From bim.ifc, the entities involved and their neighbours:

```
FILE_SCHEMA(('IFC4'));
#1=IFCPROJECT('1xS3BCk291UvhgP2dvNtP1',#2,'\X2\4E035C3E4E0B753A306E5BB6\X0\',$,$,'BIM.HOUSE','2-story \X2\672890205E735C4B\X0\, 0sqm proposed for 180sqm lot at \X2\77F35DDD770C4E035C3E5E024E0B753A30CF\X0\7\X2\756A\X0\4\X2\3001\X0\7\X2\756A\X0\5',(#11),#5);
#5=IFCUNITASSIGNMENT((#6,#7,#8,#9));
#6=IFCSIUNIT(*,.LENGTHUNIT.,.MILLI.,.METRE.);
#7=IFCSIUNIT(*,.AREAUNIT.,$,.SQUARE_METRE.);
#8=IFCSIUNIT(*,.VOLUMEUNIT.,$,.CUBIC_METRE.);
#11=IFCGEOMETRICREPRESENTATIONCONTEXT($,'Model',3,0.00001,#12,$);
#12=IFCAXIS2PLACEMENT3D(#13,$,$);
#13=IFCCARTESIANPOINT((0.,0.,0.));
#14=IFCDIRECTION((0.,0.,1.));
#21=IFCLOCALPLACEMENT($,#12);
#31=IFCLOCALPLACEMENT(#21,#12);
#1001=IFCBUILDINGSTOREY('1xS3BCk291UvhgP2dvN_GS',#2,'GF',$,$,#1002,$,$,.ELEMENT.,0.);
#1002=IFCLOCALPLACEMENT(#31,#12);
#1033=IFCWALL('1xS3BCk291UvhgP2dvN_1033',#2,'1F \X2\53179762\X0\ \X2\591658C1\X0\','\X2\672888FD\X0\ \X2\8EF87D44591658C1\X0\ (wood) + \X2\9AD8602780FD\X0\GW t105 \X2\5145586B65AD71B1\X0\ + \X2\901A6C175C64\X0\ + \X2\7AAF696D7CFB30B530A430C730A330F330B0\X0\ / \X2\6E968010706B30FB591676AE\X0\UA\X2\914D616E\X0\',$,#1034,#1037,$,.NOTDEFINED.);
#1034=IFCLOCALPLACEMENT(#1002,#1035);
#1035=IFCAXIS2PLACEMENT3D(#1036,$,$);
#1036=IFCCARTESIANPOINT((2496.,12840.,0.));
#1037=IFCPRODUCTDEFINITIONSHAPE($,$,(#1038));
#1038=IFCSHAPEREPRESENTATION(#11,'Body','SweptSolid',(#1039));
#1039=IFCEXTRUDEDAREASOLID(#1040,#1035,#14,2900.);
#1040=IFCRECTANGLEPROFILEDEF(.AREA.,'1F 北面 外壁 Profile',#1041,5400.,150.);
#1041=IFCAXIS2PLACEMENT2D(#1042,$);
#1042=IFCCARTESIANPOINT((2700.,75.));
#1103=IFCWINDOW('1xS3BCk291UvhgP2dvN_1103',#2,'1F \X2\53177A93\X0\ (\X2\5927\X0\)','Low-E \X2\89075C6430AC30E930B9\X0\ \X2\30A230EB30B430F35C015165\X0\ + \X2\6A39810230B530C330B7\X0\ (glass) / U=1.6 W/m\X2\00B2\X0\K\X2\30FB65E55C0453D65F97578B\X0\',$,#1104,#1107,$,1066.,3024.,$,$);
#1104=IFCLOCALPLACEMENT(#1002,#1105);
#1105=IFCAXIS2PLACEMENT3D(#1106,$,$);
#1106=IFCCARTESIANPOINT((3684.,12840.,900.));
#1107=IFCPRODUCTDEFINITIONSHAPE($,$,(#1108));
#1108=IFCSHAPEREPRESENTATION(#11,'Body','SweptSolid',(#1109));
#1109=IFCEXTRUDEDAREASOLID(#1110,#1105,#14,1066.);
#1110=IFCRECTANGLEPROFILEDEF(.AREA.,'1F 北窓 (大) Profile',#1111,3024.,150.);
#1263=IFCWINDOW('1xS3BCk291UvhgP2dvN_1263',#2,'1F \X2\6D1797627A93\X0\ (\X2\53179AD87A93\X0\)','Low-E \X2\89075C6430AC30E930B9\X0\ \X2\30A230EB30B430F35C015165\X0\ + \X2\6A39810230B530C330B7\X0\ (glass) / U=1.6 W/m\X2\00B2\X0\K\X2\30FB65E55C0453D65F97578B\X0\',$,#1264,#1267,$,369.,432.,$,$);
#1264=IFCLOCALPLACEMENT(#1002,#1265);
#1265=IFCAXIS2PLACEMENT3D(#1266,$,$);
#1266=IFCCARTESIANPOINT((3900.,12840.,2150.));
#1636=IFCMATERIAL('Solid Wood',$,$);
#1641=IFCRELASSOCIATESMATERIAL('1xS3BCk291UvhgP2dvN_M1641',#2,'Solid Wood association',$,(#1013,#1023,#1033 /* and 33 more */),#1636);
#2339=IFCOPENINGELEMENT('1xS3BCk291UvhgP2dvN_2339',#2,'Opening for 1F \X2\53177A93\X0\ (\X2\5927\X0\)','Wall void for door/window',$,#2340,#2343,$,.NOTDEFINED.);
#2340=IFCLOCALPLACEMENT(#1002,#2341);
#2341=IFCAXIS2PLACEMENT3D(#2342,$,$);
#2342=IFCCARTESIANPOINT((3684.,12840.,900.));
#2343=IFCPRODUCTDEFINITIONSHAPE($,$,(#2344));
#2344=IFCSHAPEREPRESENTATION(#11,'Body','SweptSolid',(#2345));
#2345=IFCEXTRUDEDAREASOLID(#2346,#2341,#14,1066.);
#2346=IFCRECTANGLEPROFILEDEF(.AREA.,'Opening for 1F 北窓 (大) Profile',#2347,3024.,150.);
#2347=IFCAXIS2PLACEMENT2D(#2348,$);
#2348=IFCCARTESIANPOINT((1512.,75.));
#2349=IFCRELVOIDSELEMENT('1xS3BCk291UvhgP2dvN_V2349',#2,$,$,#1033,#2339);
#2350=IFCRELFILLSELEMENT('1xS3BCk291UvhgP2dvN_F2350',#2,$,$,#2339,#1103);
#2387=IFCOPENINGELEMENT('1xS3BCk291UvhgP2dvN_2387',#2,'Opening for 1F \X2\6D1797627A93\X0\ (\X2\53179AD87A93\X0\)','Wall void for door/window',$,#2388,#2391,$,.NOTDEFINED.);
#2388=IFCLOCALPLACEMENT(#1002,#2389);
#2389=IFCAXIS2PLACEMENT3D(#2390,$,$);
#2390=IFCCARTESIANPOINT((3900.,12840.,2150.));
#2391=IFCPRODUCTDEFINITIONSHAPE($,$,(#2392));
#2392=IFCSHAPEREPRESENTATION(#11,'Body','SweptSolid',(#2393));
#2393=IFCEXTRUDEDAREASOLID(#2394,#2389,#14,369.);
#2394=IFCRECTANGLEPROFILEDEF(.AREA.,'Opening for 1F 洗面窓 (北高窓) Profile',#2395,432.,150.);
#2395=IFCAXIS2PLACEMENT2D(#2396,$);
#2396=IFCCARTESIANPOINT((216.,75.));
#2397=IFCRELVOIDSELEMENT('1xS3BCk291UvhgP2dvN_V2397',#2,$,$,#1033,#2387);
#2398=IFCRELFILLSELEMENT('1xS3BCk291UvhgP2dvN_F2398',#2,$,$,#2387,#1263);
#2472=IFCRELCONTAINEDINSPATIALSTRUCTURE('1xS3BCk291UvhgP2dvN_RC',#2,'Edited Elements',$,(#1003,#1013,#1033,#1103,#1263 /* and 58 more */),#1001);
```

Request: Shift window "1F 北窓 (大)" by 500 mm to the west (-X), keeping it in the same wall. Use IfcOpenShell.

```python
import ifcopenshell
import ifcopenshell.api.geometry
import ifcopenshell.util.placement

model = ifcopenshell.open("bim.ifc")

window = model.by_guid("1xS3BCk291UvhgP2dvN_1103")
opening = window.FillsVoids[0].RelatingOpeningElement
wall = opening.VoidsElements[0].RelatingBuildingElement

wall_matrix = ifcopenshell.util.placement.get_local_placement(wall.ObjectPlacement)
shift = wall_matrix[:3, 0] * -500.0
before = ifcopenshell.util.placement.get_local_placement(window.ObjectPlacement)[:3, 3].copy()

# The window is not placed relative to its opening, so move both.
for product in (opening, window):
    matrix = ifcopenshell.util.placement.get_local_placement(product.ObjectPlacement)
    matrix[:3, 3] += shift
    ifcopenshell.api.geometry.edit_object_placement(model, product=product, matrix=matrix, is_si=False)

after = ifcopenshell.util.placement.get_local_placement(window.ObjectPlacement)[:3, 3]
print("window moved by", (after - before).round(3) + 0.0)

model.write("bim_v2.ifc")
```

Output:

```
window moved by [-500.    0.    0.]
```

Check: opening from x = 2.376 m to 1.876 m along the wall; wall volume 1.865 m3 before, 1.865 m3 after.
